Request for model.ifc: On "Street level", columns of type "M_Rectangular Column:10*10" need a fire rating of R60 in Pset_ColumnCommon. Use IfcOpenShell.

First a look at what the model holds.

```python
import ifcopenshell
import ifcopenshell.util.element

model = ifcopenshell.open("model.ifc")
print(model.schema)
storey = next(s for s in model.by_type("IfcBuildingStorey") if s.Name == "Street level")
columns = [e for e in ifcopenshell.util.element.get_decomposition(storey) if e.is_a("IfcColumn")]
seen = {}
for e in columns:
    element_type = ifcopenshell.util.element.get_type(e)
    key = (element_type.Name if element_type != e and element_type else None, ifcopenshell.util.element.get_pset(e, "Pset_ColumnCommon", "FireRating"))
    seen[key] = seen.get(key, 0) + 1
for (name, value), count in sorted(seen.items(), key=str):
    print(count, "x", name, "|", value)
```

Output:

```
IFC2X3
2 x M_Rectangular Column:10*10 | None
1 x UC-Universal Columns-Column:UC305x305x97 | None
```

```python
import ifcopenshell
import ifcopenshell.api.pset
import ifcopenshell.util.element

model = ifcopenshell.open("model.ifc")

storey = next(s for s in model.by_type("IfcBuildingStorey") if s.Name == "Street level")
columns = [e for e in ifcopenshell.util.element.get_decomposition(storey) if e.is_a("IfcColumn")]

count = 0
for e in columns:
    element_type = ifcopenshell.util.element.get_type(e)
    if element_type in (None, e) or element_type.Name != "M_Rectangular Column:10*10":
        continue
    # add_pset returns the element's existing set when there is one.
    pset = ifcopenshell.api.pset.add_pset(model, product=e, name="Pset_ColumnCommon")
    ifcopenshell.api.pset.edit_pset(model, pset=pset, properties={"FireRating": "R60"})
    count += 1

print(count, "columns updated")

model.write("model_updated.ifc")
```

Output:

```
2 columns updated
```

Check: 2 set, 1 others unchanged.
